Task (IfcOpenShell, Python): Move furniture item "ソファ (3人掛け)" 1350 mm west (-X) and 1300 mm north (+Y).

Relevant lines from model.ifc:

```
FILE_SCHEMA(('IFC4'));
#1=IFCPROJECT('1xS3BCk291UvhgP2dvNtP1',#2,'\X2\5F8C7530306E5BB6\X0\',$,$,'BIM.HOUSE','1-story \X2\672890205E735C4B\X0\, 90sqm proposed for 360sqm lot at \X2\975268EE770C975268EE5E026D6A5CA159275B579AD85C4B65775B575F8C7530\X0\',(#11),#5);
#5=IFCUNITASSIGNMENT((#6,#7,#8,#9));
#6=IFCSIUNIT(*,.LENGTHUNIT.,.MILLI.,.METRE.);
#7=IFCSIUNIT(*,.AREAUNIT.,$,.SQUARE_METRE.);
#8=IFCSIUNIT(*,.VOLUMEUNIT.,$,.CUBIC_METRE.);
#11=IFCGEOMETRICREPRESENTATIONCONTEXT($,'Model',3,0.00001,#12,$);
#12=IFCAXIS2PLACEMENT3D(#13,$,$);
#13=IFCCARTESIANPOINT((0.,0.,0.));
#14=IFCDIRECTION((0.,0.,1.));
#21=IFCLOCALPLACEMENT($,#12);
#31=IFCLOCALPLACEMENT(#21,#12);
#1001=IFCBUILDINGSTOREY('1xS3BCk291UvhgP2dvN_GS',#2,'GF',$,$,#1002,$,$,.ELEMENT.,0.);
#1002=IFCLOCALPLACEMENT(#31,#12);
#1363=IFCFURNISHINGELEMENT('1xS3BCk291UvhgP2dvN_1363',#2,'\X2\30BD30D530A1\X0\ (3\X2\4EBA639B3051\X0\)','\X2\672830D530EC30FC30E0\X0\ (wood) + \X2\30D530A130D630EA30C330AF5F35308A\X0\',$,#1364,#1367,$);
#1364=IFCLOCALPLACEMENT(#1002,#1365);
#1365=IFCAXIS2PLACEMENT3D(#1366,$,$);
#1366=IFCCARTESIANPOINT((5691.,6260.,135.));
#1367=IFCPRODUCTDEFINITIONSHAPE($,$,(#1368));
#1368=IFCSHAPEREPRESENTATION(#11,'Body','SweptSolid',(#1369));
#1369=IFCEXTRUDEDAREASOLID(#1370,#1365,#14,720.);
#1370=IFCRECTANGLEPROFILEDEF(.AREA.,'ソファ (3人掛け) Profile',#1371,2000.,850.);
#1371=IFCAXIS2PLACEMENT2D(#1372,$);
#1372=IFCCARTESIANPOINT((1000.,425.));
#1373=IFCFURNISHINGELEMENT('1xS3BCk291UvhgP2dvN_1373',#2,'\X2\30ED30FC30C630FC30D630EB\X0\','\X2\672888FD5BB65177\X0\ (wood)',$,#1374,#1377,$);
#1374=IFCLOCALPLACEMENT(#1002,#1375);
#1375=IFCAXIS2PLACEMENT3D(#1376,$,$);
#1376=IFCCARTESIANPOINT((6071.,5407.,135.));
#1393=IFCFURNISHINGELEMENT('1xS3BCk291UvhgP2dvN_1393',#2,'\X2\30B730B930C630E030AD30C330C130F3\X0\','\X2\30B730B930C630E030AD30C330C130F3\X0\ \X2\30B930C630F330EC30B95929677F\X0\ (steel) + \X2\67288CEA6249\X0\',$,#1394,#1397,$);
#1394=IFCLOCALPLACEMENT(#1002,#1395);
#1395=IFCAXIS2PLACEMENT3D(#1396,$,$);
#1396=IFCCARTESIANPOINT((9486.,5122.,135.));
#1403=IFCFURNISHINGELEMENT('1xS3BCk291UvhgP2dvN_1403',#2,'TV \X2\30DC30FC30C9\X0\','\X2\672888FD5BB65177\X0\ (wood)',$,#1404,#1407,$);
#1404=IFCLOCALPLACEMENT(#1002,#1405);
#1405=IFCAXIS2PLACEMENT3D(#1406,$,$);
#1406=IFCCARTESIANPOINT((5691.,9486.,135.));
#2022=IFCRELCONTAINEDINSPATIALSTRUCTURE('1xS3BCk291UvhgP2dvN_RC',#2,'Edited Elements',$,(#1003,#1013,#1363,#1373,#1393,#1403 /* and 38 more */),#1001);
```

```python
import ifcopenshell
import ifcopenshell.api.geometry
import ifcopenshell.util.placement

model = ifcopenshell.open("model.ifc")

item = model.by_id(1363)
matrix = ifcopenshell.util.placement.get_local_placement(item.ObjectPlacement)
matrix[0, 3] -= 1350.0
matrix[1, 3] += 1300.0
ifcopenshell.api.geometry.edit_object_placement(model, product=item, matrix=matrix, is_si=False)

print(ifcopenshell.util.placement.get_local_placement(item.ObjectPlacement).round(3) + 0.0)

model.write("model-out.ifc")
```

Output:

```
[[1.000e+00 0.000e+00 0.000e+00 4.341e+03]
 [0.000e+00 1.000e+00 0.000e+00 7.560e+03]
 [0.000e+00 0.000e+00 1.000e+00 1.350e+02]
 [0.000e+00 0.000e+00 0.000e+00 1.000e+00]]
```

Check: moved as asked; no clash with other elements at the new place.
